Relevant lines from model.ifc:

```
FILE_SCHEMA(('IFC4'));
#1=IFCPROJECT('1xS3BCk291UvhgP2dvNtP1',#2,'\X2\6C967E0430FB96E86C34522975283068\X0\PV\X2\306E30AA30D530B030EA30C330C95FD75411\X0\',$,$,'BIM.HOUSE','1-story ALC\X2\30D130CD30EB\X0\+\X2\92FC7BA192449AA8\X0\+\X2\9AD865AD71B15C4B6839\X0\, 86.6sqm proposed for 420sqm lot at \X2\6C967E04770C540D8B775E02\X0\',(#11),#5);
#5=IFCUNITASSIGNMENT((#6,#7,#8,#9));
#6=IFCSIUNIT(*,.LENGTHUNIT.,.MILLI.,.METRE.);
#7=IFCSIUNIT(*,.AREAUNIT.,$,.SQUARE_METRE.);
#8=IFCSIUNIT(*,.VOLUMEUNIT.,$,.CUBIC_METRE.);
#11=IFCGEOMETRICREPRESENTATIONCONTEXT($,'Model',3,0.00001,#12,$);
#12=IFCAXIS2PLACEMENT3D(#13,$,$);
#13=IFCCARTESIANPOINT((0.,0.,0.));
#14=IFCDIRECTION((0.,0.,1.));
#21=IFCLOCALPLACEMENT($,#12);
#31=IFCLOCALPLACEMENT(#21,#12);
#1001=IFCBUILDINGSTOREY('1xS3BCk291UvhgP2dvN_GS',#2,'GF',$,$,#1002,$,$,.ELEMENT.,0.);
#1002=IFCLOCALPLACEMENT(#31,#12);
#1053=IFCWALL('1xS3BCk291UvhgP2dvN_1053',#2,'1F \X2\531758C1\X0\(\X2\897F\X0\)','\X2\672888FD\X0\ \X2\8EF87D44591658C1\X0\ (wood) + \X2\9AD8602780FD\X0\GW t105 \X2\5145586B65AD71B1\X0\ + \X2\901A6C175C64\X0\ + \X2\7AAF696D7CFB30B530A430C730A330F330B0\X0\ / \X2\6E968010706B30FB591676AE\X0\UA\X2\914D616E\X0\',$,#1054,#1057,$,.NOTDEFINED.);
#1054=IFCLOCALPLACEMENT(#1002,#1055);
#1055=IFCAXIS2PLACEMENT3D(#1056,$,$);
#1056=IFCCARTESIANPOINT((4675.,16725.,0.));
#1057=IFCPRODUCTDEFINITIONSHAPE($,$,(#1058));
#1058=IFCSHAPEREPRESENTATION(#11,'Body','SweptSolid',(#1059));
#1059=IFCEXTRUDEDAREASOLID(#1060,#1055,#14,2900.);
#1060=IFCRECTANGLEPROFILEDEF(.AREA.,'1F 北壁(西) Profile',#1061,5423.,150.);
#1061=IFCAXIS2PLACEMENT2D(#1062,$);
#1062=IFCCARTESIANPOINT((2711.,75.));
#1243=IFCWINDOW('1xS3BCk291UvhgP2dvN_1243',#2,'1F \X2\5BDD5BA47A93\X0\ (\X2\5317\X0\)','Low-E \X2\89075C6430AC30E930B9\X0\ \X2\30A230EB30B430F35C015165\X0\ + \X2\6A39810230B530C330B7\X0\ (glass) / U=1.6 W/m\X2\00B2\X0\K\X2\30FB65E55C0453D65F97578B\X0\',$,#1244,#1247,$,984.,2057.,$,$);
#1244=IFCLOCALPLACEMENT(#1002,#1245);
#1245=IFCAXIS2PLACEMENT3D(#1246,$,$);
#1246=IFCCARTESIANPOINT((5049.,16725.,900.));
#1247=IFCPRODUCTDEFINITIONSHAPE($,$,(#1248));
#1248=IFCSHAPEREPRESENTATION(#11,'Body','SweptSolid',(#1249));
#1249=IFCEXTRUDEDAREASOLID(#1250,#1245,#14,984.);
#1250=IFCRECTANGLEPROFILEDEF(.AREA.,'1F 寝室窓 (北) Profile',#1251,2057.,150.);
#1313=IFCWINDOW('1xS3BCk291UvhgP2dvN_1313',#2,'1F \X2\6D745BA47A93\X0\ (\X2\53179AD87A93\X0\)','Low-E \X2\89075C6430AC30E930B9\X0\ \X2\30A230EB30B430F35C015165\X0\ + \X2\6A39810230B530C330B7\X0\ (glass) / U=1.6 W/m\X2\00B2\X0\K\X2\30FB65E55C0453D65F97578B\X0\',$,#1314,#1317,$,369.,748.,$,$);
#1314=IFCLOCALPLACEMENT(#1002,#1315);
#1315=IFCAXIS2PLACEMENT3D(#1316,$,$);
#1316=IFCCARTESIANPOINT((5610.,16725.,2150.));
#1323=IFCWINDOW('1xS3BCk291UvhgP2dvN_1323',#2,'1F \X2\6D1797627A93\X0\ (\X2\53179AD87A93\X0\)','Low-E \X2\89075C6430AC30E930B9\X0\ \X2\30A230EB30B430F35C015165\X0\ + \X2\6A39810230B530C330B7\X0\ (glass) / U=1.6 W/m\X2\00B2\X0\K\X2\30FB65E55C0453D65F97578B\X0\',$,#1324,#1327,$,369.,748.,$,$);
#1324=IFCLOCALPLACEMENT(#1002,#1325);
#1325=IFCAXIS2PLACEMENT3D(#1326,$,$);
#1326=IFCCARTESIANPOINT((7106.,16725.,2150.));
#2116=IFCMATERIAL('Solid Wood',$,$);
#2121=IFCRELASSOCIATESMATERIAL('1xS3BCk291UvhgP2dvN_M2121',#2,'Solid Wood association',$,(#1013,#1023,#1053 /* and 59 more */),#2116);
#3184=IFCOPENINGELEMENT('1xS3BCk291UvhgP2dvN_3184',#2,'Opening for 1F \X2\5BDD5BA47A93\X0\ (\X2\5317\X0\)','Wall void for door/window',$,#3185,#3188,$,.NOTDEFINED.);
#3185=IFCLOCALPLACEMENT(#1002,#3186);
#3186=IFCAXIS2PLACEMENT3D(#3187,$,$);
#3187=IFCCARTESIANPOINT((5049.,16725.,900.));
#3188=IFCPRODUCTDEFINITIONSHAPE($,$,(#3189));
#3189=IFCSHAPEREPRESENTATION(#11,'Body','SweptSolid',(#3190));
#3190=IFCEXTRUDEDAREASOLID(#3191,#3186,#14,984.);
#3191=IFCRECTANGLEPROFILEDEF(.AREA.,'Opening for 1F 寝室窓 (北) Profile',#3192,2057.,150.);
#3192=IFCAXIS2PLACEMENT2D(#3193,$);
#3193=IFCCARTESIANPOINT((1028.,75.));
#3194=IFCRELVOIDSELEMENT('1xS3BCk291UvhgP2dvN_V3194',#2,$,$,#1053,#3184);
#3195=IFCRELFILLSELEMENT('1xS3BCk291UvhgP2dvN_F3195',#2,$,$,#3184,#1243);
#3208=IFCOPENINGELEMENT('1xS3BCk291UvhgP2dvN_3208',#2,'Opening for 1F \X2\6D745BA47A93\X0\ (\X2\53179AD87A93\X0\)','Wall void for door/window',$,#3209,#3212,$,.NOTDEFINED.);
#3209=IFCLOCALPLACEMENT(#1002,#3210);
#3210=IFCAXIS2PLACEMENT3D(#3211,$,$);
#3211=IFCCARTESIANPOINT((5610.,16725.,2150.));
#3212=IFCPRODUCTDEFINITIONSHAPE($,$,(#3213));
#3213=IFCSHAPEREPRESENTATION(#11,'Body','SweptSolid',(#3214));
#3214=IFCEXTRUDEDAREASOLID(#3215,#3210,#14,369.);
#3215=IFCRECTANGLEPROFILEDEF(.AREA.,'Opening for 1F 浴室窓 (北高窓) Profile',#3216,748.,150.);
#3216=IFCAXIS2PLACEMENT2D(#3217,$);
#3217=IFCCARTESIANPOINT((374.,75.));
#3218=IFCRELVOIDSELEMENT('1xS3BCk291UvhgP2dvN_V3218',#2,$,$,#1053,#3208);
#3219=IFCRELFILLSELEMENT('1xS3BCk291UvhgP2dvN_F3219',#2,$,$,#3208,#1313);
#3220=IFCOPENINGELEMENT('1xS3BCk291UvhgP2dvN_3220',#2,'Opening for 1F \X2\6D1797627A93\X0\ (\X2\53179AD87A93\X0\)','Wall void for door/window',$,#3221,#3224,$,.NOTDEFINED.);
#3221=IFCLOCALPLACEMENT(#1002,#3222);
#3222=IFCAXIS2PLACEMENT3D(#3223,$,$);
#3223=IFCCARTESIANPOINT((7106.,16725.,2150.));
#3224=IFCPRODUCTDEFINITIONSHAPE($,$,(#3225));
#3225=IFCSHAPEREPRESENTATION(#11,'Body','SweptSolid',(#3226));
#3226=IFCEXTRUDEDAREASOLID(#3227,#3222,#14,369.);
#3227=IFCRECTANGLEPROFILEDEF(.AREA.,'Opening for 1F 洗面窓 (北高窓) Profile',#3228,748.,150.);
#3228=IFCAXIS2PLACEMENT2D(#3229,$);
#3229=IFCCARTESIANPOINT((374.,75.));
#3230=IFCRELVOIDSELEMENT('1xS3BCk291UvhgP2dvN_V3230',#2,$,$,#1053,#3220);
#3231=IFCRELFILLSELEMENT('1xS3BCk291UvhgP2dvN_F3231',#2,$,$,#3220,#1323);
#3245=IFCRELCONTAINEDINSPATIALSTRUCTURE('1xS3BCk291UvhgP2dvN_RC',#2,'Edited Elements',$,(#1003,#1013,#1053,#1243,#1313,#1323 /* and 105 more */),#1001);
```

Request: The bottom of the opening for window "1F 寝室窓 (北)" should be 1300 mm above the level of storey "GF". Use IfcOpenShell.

```python
import numpy as np
import ifcopenshell
import ifcopenshell.api.geometry
import ifcopenshell.geom
import ifcopenshell.util.element
import ifcopenshell.util.placement
import ifcopenshell.util.shape
import ifcopenshell.util.unit

model = ifcopenshell.open("model.ifc")
unit_scale = ifcopenshell.util.unit.calculate_unit_scale(model)

window = model.by_guid("1xS3BCk291UvhgP2dvN_1243")
opening = window.FillsVoids[0].RelatingOpeningElement
storey = ifcopenshell.util.element.get_container(window, ifc_class="IfcBuildingStorey")
level = ifcopenshell.util.placement.get_local_placement(storey.ObjectPlacement)[2, 3]

# The opening's origin need not be at the sill, so measure its lowest point.
shape = ifcopenshell.geom.create_shape(ifcopenshell.geom.settings(), opening)
bottom = ifcopenshell.util.shape.get_shape_bottom_elevation(shape, shape.geometry) / unit_scale
dz = level + 1.3 / unit_scale - bottom

shift = np.array([0.0, 0.0, dz])
# The window is not placed relative to its opening, so move both.
for product in (opening, window):
    matrix = ifcopenshell.util.placement.get_local_placement(product.ObjectPlacement)
    matrix[:3, 3] += shift
    ifcopenshell.api.geometry.edit_object_placement(model, product=product, matrix=matrix, is_si=False)

print(f"moved by {dz * unit_scale:+.3f} m")

model.write("model_updated.ifc")
```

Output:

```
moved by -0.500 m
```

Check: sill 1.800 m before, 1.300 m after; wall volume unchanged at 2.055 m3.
